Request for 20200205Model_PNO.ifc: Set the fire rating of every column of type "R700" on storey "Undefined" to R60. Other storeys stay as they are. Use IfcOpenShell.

First a look at what the model holds.

```python
import ifcopenshell
import ifcopenshell.util.element

model = ifcopenshell.open("20200205Model_PNO.ifc")
print(model.schema)
storey = next(s for s in model.by_type("IfcBuildingStorey") if s.Name == "Undefined")
columns = [e for e in ifcopenshell.util.element.get_decomposition(storey) if e.is_a("IfcColumn")]
seen = {}
for e in columns:
    element_type = ifcopenshell.util.element.get_type(e)
    key = (element_type.Name if element_type != e and element_type else None, ifcopenshell.util.element.get_pset(e, "Pset_ColumnCommon", "FireRating"))
    seen[key] = seen.get(key, 0) + 1
for (name, value), count in sorted(seen.items(), key=str):
    print(count, "x", name, "|", value)
```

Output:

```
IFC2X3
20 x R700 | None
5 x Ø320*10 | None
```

```python
import ifcopenshell
import ifcopenshell.api.pset
import ifcopenshell.util.element

model = ifcopenshell.open("20200205Model_PNO.ifc")

storey = next(s for s in model.by_type("IfcBuildingStorey") if s.Name == "Undefined")
columns = [e for e in ifcopenshell.util.element.get_decomposition(storey) if e.is_a("IfcColumn")]

count = 0
for e in columns:
    element_type = ifcopenshell.util.element.get_type(e)
    if element_type in (None, e) or element_type.Name != "R700":
        continue
    found = ifcopenshell.util.element.get_pset(e, "Pset_ColumnCommon", should_inherit=False)
    if found:
        pset = model.by_id(found["id"])
        if len(ifcopenshell.util.element.get_elements_by_pset(pset)) > 1:
            pset = ifcopenshell.api.pset.unshare_pset(model, products=[e], pset=pset)[0]
    else:
        pset = ifcopenshell.api.pset.add_pset(model, product=e, name="Pset_ColumnCommon")
    ifcopenshell.api.pset.edit_pset(model, pset=pset, properties={"FireRating": "R60"})
    count += 1

print(count, "columns updated")

model.write("20200205Model_PNO_rev.ifc")
```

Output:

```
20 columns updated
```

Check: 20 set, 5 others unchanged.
